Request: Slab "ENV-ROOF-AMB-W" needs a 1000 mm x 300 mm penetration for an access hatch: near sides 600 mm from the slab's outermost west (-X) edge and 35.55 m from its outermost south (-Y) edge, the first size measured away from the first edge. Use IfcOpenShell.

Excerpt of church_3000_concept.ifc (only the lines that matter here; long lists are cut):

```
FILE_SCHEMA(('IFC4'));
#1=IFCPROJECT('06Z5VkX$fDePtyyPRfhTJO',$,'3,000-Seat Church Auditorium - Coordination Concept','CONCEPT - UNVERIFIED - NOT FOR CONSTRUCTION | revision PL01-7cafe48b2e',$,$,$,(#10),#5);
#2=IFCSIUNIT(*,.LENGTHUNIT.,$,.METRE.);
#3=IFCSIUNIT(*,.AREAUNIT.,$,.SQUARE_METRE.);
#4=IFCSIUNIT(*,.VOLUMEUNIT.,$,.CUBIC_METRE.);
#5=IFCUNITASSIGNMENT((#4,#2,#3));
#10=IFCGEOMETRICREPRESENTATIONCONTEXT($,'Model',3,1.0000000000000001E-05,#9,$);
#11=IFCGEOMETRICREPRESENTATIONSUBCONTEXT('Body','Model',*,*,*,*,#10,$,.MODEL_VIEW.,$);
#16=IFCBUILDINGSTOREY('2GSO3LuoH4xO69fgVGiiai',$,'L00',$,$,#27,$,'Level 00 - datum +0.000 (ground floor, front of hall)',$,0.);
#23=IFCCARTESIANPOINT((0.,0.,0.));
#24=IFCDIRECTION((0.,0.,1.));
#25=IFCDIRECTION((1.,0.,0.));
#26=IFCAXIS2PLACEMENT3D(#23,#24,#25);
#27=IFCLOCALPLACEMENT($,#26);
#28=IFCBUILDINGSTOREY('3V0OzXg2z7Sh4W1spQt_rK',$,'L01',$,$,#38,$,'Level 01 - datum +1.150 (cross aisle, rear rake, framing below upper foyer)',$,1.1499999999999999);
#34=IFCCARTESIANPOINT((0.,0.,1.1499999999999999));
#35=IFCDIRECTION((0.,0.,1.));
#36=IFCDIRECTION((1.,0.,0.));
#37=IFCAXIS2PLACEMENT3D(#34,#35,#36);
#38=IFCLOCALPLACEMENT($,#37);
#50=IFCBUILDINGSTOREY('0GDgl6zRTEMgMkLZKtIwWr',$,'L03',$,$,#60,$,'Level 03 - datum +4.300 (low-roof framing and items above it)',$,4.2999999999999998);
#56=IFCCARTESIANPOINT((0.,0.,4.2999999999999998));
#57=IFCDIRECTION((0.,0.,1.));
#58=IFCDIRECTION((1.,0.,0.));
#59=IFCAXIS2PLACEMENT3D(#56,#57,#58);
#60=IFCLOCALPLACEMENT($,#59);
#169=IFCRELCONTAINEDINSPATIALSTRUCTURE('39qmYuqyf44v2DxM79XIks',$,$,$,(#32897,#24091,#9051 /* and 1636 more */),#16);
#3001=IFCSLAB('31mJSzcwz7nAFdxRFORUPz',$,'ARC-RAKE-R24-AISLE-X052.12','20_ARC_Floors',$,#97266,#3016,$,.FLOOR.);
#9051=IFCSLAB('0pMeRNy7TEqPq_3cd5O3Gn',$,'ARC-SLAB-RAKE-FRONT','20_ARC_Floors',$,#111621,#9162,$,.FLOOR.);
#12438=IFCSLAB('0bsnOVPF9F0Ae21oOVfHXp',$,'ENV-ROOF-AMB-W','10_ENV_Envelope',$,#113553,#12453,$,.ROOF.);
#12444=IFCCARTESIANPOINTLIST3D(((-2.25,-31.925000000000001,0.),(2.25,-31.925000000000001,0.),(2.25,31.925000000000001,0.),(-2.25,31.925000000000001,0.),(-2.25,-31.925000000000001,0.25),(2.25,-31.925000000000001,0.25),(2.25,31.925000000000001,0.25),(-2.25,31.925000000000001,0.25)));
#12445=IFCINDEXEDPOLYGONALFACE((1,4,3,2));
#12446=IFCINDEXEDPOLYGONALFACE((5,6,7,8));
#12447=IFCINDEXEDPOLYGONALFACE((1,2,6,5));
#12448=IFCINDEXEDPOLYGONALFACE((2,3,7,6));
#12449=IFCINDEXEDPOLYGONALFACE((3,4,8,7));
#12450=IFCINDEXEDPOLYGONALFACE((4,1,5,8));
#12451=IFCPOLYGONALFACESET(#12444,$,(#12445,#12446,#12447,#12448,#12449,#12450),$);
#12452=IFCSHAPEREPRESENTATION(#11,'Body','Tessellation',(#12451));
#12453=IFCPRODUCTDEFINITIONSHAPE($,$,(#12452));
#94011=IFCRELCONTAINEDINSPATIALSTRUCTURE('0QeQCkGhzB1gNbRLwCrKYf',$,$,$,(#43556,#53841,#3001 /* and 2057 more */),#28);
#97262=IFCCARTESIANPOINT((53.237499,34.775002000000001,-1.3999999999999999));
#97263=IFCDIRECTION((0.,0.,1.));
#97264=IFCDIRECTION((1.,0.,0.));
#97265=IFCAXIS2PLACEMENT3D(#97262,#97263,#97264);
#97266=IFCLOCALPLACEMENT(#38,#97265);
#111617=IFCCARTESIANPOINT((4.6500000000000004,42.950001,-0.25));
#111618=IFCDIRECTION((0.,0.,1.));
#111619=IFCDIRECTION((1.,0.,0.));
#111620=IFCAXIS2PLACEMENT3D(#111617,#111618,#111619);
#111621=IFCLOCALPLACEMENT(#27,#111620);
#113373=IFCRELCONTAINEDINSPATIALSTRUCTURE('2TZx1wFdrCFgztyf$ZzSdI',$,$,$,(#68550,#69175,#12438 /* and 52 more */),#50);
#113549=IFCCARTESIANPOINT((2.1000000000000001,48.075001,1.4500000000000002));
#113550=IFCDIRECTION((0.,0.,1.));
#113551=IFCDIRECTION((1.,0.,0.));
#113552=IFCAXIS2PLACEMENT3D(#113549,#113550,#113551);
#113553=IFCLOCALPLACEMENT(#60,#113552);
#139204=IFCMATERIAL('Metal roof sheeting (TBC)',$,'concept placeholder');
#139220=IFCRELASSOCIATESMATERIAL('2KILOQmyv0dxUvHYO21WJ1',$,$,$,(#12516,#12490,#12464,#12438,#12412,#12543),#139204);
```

```python
import numpy as np
import ifcopenshell
import ifcopenshell.api.feature
import ifcopenshell.api.geometry
import ifcopenshell.api.root
import ifcopenshell.geom
import ifcopenshell.util.placement
import ifcopenshell.util.representation
import ifcopenshell.util.shape
import ifcopenshell.util.unit

model = ifcopenshell.open("church_3000_concept.ifc")
unit_scale = ifcopenshell.util.unit.calculate_unit_scale(model)
settings = ifcopenshell.geom.settings()


def volume(element):
    """Net volume in cubic metres, openings subtracted."""
    shape = ifcopenshell.geom.create_shape(settings, element)
    return ifcopenshell.util.shape.get_volume(shape.geometry)


slab = model.by_guid("0bsnOVPF9F0Ae21oOVfHXp")
before = volume(slab)

# Extent in the slab's own axes, in metres. The edges named are its -X and -Y sides.
slab_shape = ifcopenshell.geom.create_shape(settings, slab)
vertices = ifcopenshell.util.shape.get_vertices(slab_shape.geometry)
x_min, y_min, bottom = vertices.min(axis=0)
top = vertices[:, 2].max()

opening = ifcopenshell.api.root.create_entity(model, ifc_class="IfcOpeningElement", name="Access hatch opening", predefined_type="OPENING")
context = ifcopenshell.util.representation.get_context(model, "Model", "Body", "MODEL_VIEW")
width, depth = 1, 0.3
outline = [(0.0, 0.0), (width, 0.0), (width, depth), (0.0, depth), (0.0, 0.0)]
# Overshoot both faces by 50 mm so the cut is clean.
shape = ifcopenshell.api.geometry.add_slab_representation(
    model, context=context, depth=top - bottom + 0.1, polyline=outline
)
ifcopenshell.api.geometry.assign_representation(model, product=opening, representation=shape)

matrix = ifcopenshell.util.placement.get_local_placement(slab.ObjectPlacement)
matrix[:, 3] = matrix @ np.append(np.array([x_min + 0.6, y_min + 35.55, bottom - 0.05]) / unit_scale, 1.0)
ifcopenshell.api.geometry.edit_object_placement(model, product=opening, matrix=matrix, is_si=False)
ifcopenshell.api.feature.add_feature(model, feature=opening, element=slab)

after = volume(slab)

print(f"slab volume {before:.3f} -> {after:.3f} m3")

model.write("church_3000_concept_updated.ifc")
```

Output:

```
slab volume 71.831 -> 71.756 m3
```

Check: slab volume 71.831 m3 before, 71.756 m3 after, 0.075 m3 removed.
